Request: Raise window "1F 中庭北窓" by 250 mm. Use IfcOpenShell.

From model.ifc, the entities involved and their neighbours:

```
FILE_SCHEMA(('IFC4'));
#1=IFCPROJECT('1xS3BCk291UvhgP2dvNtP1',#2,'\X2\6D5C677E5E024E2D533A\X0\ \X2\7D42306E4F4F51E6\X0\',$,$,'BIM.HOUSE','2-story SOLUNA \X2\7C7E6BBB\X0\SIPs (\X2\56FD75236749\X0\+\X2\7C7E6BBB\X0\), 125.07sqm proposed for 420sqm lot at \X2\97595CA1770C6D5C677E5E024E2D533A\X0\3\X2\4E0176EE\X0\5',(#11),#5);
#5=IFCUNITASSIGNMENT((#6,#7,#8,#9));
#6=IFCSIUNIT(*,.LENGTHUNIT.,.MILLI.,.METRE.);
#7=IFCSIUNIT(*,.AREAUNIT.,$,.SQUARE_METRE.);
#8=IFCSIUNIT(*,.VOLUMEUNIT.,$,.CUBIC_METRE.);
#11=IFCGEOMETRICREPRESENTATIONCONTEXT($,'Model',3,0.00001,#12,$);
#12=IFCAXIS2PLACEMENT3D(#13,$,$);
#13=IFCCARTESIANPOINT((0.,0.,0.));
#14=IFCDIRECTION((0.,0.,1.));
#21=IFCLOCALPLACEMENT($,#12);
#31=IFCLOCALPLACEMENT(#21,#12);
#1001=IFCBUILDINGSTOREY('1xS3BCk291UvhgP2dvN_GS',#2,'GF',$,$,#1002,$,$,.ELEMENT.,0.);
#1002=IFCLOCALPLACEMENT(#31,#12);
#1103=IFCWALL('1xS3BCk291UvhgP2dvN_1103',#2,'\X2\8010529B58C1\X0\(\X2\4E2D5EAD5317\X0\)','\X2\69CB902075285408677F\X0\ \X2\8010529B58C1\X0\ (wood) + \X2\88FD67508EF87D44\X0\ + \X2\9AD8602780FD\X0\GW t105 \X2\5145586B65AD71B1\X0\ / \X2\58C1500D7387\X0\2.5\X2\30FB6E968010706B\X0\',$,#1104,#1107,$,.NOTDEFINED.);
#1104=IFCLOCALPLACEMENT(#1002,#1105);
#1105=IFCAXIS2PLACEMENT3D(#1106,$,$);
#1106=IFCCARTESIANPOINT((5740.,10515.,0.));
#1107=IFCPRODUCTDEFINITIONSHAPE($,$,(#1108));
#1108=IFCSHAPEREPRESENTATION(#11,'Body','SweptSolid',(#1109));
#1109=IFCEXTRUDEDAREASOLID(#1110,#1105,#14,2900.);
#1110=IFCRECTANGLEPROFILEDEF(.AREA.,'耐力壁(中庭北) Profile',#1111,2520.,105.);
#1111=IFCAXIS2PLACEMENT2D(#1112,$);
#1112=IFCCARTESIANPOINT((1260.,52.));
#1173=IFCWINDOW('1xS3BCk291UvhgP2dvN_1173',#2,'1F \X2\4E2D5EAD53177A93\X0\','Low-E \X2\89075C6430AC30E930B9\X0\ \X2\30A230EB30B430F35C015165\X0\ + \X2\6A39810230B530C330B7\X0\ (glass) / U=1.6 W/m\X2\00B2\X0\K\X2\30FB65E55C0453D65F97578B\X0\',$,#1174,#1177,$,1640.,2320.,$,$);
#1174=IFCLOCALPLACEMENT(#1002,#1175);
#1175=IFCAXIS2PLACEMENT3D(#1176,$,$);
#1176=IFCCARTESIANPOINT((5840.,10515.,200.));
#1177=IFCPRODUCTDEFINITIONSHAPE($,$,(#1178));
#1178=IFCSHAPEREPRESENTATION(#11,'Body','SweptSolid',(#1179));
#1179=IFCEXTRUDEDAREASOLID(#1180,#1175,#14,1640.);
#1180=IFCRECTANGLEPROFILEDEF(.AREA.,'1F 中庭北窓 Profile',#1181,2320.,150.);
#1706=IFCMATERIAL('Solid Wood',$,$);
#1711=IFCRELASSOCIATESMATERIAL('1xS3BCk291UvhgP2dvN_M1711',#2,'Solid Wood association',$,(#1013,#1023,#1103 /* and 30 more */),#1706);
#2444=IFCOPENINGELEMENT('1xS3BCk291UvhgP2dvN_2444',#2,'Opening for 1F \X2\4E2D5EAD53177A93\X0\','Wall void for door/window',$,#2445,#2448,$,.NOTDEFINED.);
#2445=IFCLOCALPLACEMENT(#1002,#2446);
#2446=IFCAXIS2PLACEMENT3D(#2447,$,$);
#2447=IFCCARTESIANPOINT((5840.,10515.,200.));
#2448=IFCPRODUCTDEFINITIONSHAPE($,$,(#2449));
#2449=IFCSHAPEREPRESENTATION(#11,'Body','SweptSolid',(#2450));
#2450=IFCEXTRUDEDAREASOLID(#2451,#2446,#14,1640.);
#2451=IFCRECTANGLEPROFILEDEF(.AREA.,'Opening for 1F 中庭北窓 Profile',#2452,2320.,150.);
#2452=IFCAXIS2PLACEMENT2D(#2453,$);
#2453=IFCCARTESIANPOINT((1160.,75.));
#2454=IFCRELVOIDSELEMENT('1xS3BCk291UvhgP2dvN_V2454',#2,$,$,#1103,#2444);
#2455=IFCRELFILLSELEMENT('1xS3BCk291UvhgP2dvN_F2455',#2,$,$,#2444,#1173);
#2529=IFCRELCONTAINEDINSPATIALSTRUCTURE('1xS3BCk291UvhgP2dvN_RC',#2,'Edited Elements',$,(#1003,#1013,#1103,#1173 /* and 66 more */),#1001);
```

```python
import numpy as np
import ifcopenshell
import ifcopenshell.api.geometry
import ifcopenshell.util.placement
import ifcopenshell.util.unit

model = ifcopenshell.open("model.ifc")
unit_scale = ifcopenshell.util.unit.calculate_unit_scale(model)

window = model.by_id(1173)
opening = window.FillsVoids[0].RelatingOpeningElement
dz = 250.0

shift = np.array([0.0, 0.0, dz])
# The window is not placed relative to its opening, so move both.
for product in (opening, window):
    matrix = ifcopenshell.util.placement.get_local_placement(product.ObjectPlacement)
    matrix[:3, 3] += shift
    ifcopenshell.api.geometry.edit_object_placement(model, product=product, matrix=matrix, is_si=False)

print(f"moved by {dz * unit_scale:+.3f} m")

model.write("model_updated.ifc")
```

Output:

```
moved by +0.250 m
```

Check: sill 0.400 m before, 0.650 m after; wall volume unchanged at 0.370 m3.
